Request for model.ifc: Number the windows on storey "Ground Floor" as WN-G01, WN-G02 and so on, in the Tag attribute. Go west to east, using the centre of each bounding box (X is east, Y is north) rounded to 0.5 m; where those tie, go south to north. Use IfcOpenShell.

First a look at what the model holds.

```python
import ifcopenshell
import ifcopenshell.util.element
import ifcopenshell.util.placement

model = ifcopenshell.open("model.ifc")
print(model.schema)
storey = next(s for s in model.by_type("IfcBuildingStorey") if s.Name == "Ground Floor")
windows = [e for e in ifcopenshell.util.element.get_decomposition(storey) if e.is_a("IfcWindow")]
for e in sorted(windows, key=lambda e: e.id()):
    origin = ifcopenshell.util.placement.get_local_placement(e.ObjectPlacement)[:3, 3]
    print(e.id(), e.Tag, e.Name, origin.round(2) + 0.0, sep=" | ")
```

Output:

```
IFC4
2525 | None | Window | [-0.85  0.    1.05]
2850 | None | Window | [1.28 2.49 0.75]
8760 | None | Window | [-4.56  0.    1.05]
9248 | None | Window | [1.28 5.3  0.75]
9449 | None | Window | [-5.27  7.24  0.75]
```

```python
import ifcopenshell
import ifcopenshell.geom
import ifcopenshell.util.element
import ifcopenshell.util.shape

model = ifcopenshell.open("model.ifc")
settings = ifcopenshell.geom.settings()
settings.set("use-world-coords", True)


def centre(element):
    shape = ifcopenshell.geom.create_shape(settings, element)
    return ifcopenshell.util.shape.get_bbox_centroid(shape.geometry)


storey = next(s for s in model.by_type("IfcBuildingStorey") if s.Name == "Ground Floor")
windows = [e for e in ifcopenshell.util.element.get_decomposition(storey) if e.is_a("IfcWindow")]

# Insertion points can sit at a corner or the storey origin, so sort by the geometry (in metres).
centres = {e: centre(e) for e in windows}
windows.sort(key=lambda e: (round(centres[e][0] / 0.5), centres[e][1]))

for i, e in enumerate(windows, start=1):
    number = f"WN-G{i:02d}"
    e.Tag = number
    print(e.id(), number)

model.write("model_v2.ifc")
```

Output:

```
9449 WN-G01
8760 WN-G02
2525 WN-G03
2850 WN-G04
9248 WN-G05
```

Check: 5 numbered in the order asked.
